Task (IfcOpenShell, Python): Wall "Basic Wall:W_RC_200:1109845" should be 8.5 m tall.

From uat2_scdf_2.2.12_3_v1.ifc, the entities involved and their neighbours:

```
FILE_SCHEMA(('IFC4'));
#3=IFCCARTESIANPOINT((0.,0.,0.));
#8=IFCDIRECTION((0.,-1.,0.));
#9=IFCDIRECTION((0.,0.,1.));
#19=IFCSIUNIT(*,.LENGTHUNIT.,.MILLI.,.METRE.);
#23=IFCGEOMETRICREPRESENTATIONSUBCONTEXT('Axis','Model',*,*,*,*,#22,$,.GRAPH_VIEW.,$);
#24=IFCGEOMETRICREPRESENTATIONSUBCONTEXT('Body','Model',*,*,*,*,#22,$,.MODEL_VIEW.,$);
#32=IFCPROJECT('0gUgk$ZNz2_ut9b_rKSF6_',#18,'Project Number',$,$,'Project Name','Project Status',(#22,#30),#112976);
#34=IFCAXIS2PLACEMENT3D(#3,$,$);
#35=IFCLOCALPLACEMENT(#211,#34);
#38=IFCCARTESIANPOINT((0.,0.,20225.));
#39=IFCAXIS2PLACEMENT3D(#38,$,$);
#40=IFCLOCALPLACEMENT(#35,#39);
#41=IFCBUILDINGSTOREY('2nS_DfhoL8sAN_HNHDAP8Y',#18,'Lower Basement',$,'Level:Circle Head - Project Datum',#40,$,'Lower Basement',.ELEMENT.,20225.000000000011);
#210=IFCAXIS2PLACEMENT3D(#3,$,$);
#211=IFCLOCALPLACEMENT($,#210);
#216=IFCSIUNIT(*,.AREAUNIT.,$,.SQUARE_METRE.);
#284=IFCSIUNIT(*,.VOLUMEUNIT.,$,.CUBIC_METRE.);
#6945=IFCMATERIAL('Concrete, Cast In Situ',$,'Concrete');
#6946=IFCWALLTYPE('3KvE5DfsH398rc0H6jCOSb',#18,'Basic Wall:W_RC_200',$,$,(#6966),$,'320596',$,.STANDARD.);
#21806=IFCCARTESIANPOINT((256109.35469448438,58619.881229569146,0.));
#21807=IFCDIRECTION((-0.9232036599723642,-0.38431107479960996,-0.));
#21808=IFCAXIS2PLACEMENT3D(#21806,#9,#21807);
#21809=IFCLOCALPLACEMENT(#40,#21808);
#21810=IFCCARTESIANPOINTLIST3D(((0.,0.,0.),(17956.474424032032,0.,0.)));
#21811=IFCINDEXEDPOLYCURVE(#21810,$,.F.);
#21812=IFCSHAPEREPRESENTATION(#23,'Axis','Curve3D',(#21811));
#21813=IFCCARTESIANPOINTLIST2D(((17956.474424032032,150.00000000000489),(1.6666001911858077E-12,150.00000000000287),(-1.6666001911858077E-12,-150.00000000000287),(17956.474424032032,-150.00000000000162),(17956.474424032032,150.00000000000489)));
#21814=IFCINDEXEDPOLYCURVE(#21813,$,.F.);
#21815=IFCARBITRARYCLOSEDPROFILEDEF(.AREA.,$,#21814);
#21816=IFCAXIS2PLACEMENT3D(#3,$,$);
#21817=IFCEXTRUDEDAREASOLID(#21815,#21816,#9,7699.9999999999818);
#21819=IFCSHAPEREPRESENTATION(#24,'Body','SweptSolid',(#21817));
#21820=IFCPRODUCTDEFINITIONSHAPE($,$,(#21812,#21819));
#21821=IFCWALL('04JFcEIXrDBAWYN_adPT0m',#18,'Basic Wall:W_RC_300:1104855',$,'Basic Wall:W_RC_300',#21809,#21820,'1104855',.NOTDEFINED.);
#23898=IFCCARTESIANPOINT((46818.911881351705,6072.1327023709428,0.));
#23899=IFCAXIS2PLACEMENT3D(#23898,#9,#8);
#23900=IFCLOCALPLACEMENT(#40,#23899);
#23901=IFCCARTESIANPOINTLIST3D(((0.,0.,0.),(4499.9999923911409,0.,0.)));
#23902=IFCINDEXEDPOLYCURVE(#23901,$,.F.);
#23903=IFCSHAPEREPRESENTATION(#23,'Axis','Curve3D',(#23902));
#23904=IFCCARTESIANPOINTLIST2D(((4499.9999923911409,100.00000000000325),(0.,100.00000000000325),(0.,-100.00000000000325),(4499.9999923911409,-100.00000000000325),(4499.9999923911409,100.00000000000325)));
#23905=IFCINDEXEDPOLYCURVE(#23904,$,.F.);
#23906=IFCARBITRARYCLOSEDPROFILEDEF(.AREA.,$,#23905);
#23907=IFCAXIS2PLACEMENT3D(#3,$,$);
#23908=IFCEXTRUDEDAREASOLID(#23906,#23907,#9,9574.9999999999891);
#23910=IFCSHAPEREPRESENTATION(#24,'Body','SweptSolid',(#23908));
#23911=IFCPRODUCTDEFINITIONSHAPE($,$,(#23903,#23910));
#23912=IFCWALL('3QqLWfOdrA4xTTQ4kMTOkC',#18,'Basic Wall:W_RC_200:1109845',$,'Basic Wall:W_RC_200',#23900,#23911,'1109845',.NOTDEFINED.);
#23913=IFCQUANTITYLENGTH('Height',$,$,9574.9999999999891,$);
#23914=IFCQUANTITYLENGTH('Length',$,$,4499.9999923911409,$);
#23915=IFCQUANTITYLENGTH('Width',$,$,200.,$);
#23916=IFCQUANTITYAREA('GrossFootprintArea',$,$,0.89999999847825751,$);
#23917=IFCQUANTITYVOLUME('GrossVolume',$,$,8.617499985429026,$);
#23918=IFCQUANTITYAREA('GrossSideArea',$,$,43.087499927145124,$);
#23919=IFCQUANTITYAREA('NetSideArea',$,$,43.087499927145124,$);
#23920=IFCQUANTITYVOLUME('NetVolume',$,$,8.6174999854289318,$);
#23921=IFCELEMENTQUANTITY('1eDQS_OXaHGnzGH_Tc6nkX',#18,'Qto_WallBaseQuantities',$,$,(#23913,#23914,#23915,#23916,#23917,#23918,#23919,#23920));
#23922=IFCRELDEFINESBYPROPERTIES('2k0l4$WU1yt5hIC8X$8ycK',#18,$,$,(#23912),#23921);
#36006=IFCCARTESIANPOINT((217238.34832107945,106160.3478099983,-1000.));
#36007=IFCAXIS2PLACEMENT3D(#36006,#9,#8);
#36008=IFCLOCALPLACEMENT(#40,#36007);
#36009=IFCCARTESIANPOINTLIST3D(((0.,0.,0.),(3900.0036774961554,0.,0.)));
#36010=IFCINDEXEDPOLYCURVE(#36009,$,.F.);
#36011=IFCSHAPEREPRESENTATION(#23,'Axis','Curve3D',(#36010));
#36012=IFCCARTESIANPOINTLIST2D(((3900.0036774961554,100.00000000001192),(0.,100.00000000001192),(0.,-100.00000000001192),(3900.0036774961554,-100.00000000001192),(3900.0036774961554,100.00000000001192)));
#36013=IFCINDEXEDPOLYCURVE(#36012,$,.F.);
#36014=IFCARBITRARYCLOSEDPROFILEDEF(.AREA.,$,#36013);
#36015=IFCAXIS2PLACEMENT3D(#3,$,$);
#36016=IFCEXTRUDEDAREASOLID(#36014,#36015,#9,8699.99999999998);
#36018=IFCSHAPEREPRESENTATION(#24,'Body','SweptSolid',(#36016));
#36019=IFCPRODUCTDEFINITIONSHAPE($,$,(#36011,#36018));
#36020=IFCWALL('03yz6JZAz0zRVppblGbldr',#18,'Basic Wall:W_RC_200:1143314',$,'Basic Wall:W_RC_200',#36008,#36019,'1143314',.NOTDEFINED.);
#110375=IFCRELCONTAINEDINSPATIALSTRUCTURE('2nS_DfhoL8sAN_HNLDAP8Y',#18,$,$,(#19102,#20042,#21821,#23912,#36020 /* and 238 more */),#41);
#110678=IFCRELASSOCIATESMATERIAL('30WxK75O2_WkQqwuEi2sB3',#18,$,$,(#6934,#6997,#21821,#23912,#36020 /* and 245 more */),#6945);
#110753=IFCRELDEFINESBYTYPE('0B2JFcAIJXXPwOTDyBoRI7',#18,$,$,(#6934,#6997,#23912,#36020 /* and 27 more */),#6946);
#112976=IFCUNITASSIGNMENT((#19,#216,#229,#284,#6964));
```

```python
import ifcopenshell
import ifcopenshell.api.pset
import ifcopenshell.geom
import ifcopenshell.util.element
import ifcopenshell.util.representation
import ifcopenshell.util.shape
import ifcopenshell.util.unit

model = ifcopenshell.open("uat2_scdf_2.2.12_3_v1.ifc")
unit_scale = ifcopenshell.util.unit.calculate_unit_scale(model)
area_scale = ifcopenshell.util.unit.calculate_unit_scale(model, "AREAUNIT")
volume_scale = ifcopenshell.util.unit.calculate_unit_scale(model, "VOLUMEUNIT")
settings = ifcopenshell.geom.settings()


def volume(element):
    """Net volume in cubic metres, openings subtracted."""
    shape = ifcopenshell.geom.create_shape(settings, element)
    return ifcopenshell.util.shape.get_volume(shape.geometry)


wall = model.by_guid("3QqLWfOdrA4xTTQ4kMTOkC")
before = volume(wall)

body = ifcopenshell.util.representation.get_representation(wall, "Model", "Body")
solid = body.Items[0]
old_height = solid.Depth
solid.Depth = 8.5 / unit_scale
after = volume(wall)
thickness = 0.2  # wall thickness in metres

# Update the stored height, areas and volumes.
qto = model.by_id(ifcopenshell.util.element.get_pset(wall, "Qto_WallBaseQuantities", should_inherit=False)["id"])
ifcopenshell.api.pset.edit_qto(model, qto=qto, properties={
    "Height": solid.Depth,
    "GrossVolume": ifcopenshell.util.element.get_pset(wall, "Qto_WallBaseQuantities", "GrossVolume") * solid.Depth / old_height,
    "GrossSideArea": ifcopenshell.util.element.get_pset(wall, "Qto_WallBaseQuantities", "GrossSideArea") * solid.Depth / old_height,
    "NetSideArea": after / thickness / area_scale,
    "NetVolume": after / volume_scale,
})

print(f"height {old_height:g} -> {solid.Depth:g}, volume {before:.3f} -> {after:.3f} m3")

model.write("uat2_scdf_2.2.12_3_v1_rev.ifc")
```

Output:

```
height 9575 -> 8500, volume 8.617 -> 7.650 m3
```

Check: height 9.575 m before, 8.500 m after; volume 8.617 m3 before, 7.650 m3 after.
